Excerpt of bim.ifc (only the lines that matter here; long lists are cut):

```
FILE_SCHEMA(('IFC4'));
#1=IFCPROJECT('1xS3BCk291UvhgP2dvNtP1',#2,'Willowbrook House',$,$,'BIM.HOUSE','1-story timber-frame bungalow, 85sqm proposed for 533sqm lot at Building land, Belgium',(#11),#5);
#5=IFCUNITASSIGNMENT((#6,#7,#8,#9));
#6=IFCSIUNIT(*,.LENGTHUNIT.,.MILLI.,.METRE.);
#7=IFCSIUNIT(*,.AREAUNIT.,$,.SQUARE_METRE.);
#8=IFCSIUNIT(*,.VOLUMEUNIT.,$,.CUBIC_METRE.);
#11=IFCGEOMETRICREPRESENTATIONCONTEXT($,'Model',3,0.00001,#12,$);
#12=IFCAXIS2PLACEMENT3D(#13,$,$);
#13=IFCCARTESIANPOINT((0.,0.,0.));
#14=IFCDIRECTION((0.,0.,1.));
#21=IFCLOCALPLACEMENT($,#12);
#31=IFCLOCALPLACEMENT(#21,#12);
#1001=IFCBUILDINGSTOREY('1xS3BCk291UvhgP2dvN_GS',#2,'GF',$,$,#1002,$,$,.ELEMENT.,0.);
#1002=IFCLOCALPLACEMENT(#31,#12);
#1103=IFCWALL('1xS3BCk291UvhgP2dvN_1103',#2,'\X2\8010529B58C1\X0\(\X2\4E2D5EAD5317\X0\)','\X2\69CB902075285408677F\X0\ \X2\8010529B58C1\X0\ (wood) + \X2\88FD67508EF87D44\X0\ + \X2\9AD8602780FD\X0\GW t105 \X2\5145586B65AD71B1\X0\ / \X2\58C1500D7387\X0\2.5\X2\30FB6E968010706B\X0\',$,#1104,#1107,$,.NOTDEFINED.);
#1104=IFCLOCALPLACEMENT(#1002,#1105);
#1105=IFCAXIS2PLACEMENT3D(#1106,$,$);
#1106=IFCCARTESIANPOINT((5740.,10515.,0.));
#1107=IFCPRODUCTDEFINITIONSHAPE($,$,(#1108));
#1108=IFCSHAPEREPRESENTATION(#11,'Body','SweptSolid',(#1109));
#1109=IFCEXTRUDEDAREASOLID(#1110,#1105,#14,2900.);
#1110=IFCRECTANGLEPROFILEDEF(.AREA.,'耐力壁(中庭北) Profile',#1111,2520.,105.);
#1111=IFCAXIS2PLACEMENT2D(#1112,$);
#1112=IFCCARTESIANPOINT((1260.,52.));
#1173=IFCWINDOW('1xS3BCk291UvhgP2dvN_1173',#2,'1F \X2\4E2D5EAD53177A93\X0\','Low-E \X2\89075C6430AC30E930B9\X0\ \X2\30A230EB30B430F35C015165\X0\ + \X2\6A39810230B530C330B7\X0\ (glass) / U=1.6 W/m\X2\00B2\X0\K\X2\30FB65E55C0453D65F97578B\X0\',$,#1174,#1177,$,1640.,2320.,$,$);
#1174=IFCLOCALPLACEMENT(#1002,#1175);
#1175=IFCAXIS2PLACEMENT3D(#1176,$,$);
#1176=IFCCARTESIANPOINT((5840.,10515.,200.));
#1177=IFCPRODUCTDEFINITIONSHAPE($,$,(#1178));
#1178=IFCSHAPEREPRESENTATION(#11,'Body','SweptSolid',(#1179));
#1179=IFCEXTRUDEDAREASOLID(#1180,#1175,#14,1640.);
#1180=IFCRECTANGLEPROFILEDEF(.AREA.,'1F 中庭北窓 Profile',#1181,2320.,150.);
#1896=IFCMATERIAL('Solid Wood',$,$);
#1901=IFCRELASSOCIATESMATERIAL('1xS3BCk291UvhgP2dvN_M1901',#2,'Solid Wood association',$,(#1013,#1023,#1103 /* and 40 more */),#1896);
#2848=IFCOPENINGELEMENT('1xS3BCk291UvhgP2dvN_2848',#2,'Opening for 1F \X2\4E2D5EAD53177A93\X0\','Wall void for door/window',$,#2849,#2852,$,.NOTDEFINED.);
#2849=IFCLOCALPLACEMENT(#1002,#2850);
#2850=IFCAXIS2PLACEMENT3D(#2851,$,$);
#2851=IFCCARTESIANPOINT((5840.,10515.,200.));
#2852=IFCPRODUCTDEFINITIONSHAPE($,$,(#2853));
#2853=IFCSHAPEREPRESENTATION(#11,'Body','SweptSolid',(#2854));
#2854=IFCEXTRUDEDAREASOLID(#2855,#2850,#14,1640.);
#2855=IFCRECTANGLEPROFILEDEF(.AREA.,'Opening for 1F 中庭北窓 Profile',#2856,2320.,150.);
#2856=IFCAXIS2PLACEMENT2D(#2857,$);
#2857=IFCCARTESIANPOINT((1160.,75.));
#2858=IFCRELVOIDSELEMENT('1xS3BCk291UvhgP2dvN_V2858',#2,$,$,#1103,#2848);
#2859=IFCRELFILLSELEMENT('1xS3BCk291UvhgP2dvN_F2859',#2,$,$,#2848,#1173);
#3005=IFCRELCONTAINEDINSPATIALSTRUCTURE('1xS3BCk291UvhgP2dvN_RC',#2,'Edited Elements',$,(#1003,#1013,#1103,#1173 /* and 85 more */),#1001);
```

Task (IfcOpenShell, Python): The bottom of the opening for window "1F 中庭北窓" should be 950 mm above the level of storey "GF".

```python
import numpy as np
import ifcopenshell
import ifcopenshell.api.geometry
import ifcopenshell.geom
import ifcopenshell.util.element
import ifcopenshell.util.placement
import ifcopenshell.util.shape
import ifcopenshell.util.unit

model = ifcopenshell.open("bim.ifc")
unit_scale = ifcopenshell.util.unit.calculate_unit_scale(model)

window = model.by_guid("1xS3BCk291UvhgP2dvN_1173")
opening = window.FillsVoids[0].RelatingOpeningElement
storey = ifcopenshell.util.element.get_container(window, ifc_class="IfcBuildingStorey")
level = ifcopenshell.util.placement.get_local_placement(storey.ObjectPlacement)[2, 3]

# The opening's origin need not be at the sill, so measure its lowest point.
shape = ifcopenshell.geom.create_shape(ifcopenshell.geom.settings(), opening)
bottom = ifcopenshell.util.shape.get_shape_bottom_elevation(shape, shape.geometry) / unit_scale
dz = level + 0.95 / unit_scale - bottom

shift = np.array([0.0, 0.0, dz])
# The window is not placed relative to its opening, so move both.
for product in (opening, window):
    matrix = ifcopenshell.util.placement.get_local_placement(product.ObjectPlacement)
    matrix[:3, 3] += shift
    ifcopenshell.api.geometry.edit_object_placement(model, product=product, matrix=matrix, is_si=False)

print(f"moved by {dz * unit_scale:+.3f} m")

model.write("bim_edited.ifc")
```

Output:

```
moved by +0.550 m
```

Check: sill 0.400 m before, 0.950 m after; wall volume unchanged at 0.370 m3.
